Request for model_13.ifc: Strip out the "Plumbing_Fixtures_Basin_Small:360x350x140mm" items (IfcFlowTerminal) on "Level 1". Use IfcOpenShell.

First a look at what the model holds.

```python
import ifcopenshell
import ifcopenshell.util.element

model = ifcopenshell.open("model_13.ifc")
print(model.schema)
storey = next(s for s in model.by_type("IfcBuildingStorey") if s.Name == "Level 1")
terminals = [e for e in ifcopenshell.util.element.get_decomposition(storey) if e.is_a("IfcFlowTerminal")]
seen = {}
for e in terminals:
    element_type = ifcopenshell.util.element.get_type(e)
    name = element_type.Name if element_type not in (None, e) else None
    seen[name] = seen.get(name, 0) + 1
for name, count in sorted(seen.items(), key=str):
    print(count, "x", name)
```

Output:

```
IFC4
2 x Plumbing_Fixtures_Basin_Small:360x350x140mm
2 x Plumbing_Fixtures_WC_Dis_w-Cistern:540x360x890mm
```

```python
import ifcopenshell
import ifcopenshell.api.root
import ifcopenshell.util.element

model = ifcopenshell.open("model_13.ifc")

storey = next(s for s in model.by_type("IfcBuildingStorey") if s.Name == "Level 1")
terminals = [e for e in ifcopenshell.util.element.get_decomposition(storey) if e.is_a("IfcFlowTerminal")]
targets = [e for e in terminals if (t := ifcopenshell.util.element.get_type(e)) not in (None, e) and t.Name == "Plumbing_Fixtures_Basin_Small:360x350x140mm"]

for e in targets:
    ifcopenshell.api.root.remove_product(model, product=e)
print(len(targets), "removed")

model.write("model_13_v2.ifc")
```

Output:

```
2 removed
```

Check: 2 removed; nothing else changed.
